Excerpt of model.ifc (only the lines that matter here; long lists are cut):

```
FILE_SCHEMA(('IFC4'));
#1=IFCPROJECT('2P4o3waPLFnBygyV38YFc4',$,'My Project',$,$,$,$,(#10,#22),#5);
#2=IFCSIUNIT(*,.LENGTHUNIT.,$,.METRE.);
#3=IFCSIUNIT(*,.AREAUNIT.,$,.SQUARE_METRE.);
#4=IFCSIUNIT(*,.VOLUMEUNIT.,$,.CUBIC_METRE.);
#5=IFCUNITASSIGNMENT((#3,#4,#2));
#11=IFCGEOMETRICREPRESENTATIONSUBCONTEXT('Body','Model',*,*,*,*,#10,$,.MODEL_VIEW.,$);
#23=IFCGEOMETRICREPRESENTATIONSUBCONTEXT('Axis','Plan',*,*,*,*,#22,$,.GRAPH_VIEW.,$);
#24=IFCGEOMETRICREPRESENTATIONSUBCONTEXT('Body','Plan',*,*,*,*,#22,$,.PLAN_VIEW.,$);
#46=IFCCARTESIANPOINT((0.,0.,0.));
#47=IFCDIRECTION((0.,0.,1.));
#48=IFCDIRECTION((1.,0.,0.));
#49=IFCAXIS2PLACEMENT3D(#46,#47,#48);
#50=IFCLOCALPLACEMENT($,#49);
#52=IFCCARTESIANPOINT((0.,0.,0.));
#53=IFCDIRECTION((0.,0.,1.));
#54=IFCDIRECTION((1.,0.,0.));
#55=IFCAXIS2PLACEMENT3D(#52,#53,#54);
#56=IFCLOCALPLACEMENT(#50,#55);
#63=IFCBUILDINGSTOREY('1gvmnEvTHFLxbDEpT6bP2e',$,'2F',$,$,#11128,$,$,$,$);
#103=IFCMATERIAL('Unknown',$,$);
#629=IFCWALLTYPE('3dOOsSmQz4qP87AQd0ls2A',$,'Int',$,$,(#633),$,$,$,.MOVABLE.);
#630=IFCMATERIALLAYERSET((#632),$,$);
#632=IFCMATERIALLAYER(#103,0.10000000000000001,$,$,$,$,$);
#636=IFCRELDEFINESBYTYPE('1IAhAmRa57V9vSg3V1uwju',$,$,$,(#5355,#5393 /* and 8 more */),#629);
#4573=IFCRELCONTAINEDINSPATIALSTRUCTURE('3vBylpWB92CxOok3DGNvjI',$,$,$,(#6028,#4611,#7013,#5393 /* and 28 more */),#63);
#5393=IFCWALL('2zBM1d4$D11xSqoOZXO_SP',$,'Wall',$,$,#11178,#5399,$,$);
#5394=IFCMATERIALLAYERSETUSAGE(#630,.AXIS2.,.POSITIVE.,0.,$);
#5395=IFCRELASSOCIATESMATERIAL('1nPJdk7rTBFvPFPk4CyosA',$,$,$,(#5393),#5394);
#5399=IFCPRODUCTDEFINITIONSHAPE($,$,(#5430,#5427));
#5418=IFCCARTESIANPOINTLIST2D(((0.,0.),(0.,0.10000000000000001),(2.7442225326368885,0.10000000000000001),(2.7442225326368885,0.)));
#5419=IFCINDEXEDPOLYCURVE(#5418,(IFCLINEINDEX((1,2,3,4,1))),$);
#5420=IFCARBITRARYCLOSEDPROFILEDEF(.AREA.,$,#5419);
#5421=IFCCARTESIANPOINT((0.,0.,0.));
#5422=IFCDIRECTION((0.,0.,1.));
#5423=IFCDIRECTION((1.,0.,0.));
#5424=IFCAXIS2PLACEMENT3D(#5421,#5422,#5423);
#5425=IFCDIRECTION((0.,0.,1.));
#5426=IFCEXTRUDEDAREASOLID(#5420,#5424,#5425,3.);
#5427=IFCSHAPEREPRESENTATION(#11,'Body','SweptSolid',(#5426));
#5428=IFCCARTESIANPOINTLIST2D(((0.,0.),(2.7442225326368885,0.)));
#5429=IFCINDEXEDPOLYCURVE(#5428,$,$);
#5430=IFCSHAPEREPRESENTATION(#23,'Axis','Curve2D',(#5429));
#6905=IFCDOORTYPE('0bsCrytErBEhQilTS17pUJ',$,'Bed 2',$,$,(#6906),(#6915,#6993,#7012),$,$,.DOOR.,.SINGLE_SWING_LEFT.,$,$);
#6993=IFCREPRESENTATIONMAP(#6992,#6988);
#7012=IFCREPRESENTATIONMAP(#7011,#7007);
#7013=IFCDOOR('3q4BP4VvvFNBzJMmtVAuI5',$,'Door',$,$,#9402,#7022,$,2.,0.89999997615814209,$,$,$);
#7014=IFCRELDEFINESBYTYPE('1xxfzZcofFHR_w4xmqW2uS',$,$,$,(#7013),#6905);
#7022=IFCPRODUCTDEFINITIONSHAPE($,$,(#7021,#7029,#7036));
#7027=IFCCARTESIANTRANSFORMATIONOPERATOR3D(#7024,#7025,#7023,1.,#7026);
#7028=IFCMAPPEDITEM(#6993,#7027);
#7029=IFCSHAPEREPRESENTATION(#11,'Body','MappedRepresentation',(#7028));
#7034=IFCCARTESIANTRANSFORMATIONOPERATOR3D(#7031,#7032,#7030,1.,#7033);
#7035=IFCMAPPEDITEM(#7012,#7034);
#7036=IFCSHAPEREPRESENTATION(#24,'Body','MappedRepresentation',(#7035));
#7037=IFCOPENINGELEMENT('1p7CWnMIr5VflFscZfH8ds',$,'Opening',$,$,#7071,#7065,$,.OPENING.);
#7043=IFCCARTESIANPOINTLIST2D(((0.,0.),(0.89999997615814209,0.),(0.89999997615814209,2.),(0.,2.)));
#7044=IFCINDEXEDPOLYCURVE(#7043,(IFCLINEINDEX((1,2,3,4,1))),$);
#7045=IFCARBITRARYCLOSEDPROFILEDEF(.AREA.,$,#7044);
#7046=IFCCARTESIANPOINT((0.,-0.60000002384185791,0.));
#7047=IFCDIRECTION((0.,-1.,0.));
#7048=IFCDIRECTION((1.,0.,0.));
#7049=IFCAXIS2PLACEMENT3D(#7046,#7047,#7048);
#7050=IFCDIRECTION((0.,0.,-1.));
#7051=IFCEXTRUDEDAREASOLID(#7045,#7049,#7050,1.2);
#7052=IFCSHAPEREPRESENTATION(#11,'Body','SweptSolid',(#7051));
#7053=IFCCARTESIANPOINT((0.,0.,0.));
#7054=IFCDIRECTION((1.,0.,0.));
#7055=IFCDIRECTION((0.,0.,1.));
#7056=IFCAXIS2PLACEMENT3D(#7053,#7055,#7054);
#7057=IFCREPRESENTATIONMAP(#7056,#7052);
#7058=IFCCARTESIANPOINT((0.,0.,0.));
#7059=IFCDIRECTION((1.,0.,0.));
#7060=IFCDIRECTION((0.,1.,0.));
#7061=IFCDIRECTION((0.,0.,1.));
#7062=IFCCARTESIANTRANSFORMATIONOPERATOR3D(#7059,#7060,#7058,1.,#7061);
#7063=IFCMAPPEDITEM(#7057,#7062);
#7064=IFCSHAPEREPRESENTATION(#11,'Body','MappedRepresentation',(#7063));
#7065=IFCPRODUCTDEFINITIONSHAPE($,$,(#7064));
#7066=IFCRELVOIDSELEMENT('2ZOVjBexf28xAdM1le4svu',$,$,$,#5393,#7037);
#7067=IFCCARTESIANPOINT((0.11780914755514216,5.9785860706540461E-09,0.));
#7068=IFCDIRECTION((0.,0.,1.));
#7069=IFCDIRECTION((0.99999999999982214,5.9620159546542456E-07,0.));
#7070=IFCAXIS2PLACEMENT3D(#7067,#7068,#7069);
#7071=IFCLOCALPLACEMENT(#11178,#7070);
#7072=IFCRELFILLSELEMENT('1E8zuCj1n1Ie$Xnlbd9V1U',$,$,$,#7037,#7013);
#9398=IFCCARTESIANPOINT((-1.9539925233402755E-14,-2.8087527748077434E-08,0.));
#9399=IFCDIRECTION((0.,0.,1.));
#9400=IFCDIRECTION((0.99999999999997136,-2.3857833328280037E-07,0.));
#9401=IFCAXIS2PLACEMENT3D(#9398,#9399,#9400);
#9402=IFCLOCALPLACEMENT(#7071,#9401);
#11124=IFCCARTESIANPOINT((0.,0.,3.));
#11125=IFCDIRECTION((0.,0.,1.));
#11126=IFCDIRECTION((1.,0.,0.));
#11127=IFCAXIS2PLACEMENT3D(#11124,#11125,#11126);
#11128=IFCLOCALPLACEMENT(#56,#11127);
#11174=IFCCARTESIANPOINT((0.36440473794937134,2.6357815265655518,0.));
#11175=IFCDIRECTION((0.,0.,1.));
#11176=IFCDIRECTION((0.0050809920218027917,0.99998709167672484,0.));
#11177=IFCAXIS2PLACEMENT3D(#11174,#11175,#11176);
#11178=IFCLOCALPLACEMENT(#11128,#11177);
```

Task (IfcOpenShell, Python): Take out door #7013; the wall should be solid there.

```python
import ifcopenshell
import ifcopenshell.api.feature
import ifcopenshell.api.root
import ifcopenshell.geom
import ifcopenshell.util.shape

model = ifcopenshell.open("model.ifc")
settings = ifcopenshell.geom.settings()


def volume(element):
    """Net volume in cubic metres, openings subtracted."""
    shape = ifcopenshell.geom.create_shape(settings, element)
    return ifcopenshell.util.shape.get_volume(shape.geometry)


door = model.by_guid("3q4BP4VvvFNBzJMmtVAuI5")
opening = door.FillsVoids[0].RelatingOpeningElement
wall = opening.VoidsElements[0].RelatingBuildingElement
before = volume(wall)

ifcopenshell.api.root.remove_product(model, product=door)
ifcopenshell.api.feature.remove_feature(model, feature=opening)

after = volume(wall)

print(f"wall volume {before:.3f} -> {after:.3f} m3")

model.write("model_v2.ifc")
```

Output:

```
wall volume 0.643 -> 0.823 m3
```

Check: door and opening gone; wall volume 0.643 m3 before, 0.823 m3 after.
